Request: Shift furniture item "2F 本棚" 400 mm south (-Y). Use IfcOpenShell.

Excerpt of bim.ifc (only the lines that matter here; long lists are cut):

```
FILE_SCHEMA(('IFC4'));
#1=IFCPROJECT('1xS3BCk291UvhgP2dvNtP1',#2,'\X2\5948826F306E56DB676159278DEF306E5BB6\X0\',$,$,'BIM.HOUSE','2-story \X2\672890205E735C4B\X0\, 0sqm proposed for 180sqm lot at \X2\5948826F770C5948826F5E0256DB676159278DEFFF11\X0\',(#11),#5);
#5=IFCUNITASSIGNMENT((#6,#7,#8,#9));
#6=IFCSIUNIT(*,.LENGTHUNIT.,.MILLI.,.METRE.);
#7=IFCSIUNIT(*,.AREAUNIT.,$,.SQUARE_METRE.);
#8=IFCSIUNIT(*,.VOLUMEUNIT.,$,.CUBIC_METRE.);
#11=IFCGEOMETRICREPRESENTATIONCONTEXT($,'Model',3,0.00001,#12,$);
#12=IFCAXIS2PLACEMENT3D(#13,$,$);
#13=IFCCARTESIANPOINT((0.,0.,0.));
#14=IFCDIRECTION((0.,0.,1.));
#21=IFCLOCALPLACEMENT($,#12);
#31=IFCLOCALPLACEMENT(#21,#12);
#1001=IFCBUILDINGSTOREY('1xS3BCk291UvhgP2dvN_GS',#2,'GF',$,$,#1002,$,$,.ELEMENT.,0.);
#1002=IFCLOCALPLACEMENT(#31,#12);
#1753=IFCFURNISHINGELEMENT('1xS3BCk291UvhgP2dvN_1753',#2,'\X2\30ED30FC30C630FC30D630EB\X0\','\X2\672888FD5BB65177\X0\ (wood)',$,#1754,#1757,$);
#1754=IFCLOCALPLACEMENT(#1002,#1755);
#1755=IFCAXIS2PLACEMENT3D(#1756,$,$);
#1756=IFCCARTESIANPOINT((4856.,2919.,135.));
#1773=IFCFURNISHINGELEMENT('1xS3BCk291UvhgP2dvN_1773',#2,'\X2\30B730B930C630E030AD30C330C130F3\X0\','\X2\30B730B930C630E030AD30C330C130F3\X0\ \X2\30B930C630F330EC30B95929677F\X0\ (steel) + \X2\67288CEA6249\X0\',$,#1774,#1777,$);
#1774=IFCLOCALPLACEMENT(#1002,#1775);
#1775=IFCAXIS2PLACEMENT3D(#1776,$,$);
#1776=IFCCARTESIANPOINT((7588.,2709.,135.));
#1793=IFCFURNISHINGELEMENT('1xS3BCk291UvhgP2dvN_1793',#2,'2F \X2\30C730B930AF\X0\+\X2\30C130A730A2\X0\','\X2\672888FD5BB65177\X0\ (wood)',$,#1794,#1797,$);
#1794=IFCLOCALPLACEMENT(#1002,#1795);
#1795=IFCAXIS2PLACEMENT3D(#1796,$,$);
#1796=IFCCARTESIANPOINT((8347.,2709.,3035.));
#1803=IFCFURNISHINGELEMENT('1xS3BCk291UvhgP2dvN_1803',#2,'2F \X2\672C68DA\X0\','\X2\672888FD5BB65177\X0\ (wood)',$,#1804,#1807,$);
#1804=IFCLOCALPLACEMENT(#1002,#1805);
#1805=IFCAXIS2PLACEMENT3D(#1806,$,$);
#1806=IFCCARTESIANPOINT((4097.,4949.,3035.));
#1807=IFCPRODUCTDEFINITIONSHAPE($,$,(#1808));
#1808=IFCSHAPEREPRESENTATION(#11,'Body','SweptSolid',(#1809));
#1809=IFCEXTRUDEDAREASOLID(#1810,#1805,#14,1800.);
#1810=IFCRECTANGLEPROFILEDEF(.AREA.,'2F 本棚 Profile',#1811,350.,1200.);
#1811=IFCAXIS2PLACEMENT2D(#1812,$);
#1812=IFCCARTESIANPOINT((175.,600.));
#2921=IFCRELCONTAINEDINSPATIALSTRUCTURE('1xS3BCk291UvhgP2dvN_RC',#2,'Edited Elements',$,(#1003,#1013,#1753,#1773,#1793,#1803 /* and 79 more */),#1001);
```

```python
import ifcopenshell
import ifcopenshell.api.geometry
import ifcopenshell.util.placement
import ifcopenshell.util.unit

model = ifcopenshell.open("bim.ifc")
unit_scale = ifcopenshell.util.unit.calculate_unit_scale(model)

item = model.by_guid("1xS3BCk291UvhgP2dvN_1803")
matrix = ifcopenshell.util.placement.get_local_placement(item.ObjectPlacement)
matrix[1, 3] -= 0.4 / unit_scale
ifcopenshell.api.geometry.edit_object_placement(model, product=item, matrix=matrix, is_si=False)

print(ifcopenshell.util.placement.get_local_placement(item.ObjectPlacement).round(3) + 0.0)

model.write("bim_updated.ifc")
```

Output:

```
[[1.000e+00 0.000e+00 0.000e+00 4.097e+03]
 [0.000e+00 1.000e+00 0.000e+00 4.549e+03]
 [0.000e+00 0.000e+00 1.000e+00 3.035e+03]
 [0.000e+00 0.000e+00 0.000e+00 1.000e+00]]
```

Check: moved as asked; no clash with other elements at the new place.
